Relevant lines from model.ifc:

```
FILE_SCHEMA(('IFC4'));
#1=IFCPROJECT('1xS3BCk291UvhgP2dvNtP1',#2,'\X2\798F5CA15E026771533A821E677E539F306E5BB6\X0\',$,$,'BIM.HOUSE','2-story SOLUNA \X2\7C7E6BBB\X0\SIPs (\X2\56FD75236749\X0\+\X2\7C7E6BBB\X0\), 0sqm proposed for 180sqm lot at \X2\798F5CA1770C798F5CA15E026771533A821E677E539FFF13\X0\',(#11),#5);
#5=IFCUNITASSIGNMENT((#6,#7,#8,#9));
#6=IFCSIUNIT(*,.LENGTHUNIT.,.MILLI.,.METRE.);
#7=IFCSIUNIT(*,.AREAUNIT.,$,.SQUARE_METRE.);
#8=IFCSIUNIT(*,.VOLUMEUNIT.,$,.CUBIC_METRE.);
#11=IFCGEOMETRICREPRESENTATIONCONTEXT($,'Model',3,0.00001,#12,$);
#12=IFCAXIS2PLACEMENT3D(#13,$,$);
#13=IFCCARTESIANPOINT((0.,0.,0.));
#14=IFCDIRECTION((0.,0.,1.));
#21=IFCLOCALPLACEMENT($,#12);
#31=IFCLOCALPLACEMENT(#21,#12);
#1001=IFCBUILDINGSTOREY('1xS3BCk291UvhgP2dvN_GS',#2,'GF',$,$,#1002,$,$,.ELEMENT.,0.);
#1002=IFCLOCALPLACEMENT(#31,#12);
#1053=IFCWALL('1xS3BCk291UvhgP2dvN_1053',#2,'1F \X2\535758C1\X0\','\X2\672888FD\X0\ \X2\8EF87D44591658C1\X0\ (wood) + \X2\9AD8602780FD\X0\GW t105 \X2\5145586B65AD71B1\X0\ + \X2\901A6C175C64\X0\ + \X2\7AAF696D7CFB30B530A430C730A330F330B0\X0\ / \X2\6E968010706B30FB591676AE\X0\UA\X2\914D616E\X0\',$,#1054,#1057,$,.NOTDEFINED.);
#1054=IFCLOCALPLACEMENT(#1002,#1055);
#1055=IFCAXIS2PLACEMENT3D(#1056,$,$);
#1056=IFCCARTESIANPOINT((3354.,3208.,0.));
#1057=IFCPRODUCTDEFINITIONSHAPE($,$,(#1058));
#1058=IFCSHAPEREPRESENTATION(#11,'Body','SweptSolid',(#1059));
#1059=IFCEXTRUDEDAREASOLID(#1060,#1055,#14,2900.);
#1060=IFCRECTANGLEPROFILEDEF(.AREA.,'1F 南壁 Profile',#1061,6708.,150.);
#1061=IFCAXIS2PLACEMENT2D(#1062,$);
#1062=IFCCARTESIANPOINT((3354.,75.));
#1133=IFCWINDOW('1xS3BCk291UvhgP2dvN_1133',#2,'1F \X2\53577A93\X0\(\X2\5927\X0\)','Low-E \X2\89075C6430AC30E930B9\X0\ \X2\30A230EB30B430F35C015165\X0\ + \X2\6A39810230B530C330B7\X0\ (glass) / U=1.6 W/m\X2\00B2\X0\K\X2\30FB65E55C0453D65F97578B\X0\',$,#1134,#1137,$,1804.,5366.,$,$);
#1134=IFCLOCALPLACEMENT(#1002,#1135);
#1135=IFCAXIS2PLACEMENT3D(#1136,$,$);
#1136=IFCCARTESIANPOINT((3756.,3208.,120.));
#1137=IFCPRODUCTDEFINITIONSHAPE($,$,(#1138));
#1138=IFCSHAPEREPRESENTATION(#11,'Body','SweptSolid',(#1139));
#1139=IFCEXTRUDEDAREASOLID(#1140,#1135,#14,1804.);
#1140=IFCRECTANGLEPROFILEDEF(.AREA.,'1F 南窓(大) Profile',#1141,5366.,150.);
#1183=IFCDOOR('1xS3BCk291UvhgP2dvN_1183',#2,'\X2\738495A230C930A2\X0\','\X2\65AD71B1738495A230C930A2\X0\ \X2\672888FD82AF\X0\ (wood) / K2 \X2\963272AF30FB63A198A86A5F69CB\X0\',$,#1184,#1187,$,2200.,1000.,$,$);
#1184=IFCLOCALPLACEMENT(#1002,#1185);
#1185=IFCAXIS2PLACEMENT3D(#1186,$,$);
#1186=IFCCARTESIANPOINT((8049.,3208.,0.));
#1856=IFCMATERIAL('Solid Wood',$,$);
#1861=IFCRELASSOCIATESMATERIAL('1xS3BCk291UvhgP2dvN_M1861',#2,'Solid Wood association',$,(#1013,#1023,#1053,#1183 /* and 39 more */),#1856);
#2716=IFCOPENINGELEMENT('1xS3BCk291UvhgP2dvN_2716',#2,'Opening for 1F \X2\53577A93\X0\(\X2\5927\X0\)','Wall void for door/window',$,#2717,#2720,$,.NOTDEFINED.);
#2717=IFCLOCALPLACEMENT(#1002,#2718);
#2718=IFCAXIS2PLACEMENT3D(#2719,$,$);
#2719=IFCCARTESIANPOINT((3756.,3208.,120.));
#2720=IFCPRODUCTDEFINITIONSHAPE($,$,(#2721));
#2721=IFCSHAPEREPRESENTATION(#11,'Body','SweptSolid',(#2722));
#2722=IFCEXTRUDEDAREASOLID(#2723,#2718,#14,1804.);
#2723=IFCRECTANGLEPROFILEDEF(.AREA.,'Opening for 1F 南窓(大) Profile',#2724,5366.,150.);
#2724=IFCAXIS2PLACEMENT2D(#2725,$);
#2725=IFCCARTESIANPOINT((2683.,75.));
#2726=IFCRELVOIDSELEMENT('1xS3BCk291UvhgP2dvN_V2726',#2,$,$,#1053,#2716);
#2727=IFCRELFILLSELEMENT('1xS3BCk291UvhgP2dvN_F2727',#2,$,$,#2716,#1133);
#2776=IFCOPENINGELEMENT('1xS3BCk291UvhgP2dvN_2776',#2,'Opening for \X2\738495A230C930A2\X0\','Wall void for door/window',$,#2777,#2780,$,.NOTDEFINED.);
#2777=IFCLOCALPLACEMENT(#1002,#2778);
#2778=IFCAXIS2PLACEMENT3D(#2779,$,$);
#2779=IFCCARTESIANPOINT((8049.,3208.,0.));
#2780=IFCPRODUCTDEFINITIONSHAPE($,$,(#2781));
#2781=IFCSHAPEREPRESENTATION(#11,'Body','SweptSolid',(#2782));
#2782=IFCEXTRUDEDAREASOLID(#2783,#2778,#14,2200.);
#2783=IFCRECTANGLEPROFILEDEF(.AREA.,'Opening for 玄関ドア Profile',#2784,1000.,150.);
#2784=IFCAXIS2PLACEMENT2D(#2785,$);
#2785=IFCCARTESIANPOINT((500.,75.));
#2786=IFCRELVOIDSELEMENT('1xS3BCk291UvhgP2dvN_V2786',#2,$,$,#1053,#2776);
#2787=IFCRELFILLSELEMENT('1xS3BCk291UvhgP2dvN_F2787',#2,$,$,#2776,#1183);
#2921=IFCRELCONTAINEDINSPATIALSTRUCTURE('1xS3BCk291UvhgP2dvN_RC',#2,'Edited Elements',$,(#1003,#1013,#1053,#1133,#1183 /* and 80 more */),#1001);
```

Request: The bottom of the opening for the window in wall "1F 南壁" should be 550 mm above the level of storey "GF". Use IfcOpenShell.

```python
import numpy as np
import ifcopenshell
import ifcopenshell.api.geometry
import ifcopenshell.geom
import ifcopenshell.util.element
import ifcopenshell.util.placement
import ifcopenshell.util.shape
import ifcopenshell.util.unit

model = ifcopenshell.open("model.ifc")
unit_scale = ifcopenshell.util.unit.calculate_unit_scale(model)

window = model.by_guid("1xS3BCk291UvhgP2dvN_1133")
opening = window.FillsVoids[0].RelatingOpeningElement
storey = ifcopenshell.util.element.get_container(window, ifc_class="IfcBuildingStorey")
level = ifcopenshell.util.placement.get_local_placement(storey.ObjectPlacement)[2, 3]

# The opening's origin need not be at the sill, so measure its lowest point.
shape = ifcopenshell.geom.create_shape(ifcopenshell.geom.settings(), opening)
bottom = ifcopenshell.util.shape.get_shape_bottom_elevation(shape, shape.geometry) / unit_scale
dz = level + 0.55 / unit_scale - bottom

shift = np.array([0.0, 0.0, dz])
# The window is not placed relative to its opening, so move both.
for product in (opening, window):
    matrix = ifcopenshell.util.placement.get_local_placement(product.ObjectPlacement)
    matrix[:3, 3] += shift
    ifcopenshell.api.geometry.edit_object_placement(model, product=product, matrix=matrix, is_si=False)

print(f"moved by {dz * unit_scale:+.3f} m")

model.write("model_rev.ifc")
```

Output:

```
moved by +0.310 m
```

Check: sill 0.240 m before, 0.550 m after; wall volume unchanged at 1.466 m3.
